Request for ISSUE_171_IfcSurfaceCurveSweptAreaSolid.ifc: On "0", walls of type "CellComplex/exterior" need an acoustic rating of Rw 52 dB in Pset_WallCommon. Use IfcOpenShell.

First a look at what the model holds.

```python
import ifcopenshell
import ifcopenshell.util.element

model = ifcopenshell.open("ISSUE_171_IfcSurfaceCurveSweptAreaSolid.ifc")
print(model.schema)
storey = next(s for s in model.by_type("IfcBuildingStorey") if s.Name == "0")
walls = [e for e in ifcopenshell.util.element.get_decomposition(storey) if e.is_a("IfcWall")]
seen = {}
for e in walls:
    element_type = ifcopenshell.util.element.get_type(e)
    key = (element_type.Name if element_type != e and element_type else None, ifcopenshell.util.element.get_pset(e, "Pset_WallCommon", "AcousticRating"))
    seen[key] = seen.get(key, 0) + 1
for (name, value), count in sorted(seen.items(), key=str):
    print(count, "x", name, "|", value)
```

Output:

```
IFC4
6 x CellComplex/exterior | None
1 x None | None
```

```python
import ifcopenshell
import ifcopenshell.api.pset
import ifcopenshell.util.element

model = ifcopenshell.open("ISSUE_171_IfcSurfaceCurveSweptAreaSolid.ifc")

storey = next(s for s in model.by_type("IfcBuildingStorey") if s.Name == "0")
walls = [e for e in ifcopenshell.util.element.get_decomposition(storey) if e.is_a("IfcWall")]

count = 0
for e in walls:
    element_type = ifcopenshell.util.element.get_type(e)
    if element_type in (None, e) or element_type.Name != "CellComplex/exterior":
        continue
    # add_pset returns the element's existing set when there is one.
    pset = ifcopenshell.api.pset.add_pset(model, product=e, name="Pset_WallCommon")
    ifcopenshell.api.pset.edit_pset(model, pset=pset, properties={"AcousticRating": "Rw 52 dB"})
    count += 1

print(count, "walls updated")

model.write("ISSUE_171_IfcSurfaceCurveSweptAreaSolid_edited.ifc")
```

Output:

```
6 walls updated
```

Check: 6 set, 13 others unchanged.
